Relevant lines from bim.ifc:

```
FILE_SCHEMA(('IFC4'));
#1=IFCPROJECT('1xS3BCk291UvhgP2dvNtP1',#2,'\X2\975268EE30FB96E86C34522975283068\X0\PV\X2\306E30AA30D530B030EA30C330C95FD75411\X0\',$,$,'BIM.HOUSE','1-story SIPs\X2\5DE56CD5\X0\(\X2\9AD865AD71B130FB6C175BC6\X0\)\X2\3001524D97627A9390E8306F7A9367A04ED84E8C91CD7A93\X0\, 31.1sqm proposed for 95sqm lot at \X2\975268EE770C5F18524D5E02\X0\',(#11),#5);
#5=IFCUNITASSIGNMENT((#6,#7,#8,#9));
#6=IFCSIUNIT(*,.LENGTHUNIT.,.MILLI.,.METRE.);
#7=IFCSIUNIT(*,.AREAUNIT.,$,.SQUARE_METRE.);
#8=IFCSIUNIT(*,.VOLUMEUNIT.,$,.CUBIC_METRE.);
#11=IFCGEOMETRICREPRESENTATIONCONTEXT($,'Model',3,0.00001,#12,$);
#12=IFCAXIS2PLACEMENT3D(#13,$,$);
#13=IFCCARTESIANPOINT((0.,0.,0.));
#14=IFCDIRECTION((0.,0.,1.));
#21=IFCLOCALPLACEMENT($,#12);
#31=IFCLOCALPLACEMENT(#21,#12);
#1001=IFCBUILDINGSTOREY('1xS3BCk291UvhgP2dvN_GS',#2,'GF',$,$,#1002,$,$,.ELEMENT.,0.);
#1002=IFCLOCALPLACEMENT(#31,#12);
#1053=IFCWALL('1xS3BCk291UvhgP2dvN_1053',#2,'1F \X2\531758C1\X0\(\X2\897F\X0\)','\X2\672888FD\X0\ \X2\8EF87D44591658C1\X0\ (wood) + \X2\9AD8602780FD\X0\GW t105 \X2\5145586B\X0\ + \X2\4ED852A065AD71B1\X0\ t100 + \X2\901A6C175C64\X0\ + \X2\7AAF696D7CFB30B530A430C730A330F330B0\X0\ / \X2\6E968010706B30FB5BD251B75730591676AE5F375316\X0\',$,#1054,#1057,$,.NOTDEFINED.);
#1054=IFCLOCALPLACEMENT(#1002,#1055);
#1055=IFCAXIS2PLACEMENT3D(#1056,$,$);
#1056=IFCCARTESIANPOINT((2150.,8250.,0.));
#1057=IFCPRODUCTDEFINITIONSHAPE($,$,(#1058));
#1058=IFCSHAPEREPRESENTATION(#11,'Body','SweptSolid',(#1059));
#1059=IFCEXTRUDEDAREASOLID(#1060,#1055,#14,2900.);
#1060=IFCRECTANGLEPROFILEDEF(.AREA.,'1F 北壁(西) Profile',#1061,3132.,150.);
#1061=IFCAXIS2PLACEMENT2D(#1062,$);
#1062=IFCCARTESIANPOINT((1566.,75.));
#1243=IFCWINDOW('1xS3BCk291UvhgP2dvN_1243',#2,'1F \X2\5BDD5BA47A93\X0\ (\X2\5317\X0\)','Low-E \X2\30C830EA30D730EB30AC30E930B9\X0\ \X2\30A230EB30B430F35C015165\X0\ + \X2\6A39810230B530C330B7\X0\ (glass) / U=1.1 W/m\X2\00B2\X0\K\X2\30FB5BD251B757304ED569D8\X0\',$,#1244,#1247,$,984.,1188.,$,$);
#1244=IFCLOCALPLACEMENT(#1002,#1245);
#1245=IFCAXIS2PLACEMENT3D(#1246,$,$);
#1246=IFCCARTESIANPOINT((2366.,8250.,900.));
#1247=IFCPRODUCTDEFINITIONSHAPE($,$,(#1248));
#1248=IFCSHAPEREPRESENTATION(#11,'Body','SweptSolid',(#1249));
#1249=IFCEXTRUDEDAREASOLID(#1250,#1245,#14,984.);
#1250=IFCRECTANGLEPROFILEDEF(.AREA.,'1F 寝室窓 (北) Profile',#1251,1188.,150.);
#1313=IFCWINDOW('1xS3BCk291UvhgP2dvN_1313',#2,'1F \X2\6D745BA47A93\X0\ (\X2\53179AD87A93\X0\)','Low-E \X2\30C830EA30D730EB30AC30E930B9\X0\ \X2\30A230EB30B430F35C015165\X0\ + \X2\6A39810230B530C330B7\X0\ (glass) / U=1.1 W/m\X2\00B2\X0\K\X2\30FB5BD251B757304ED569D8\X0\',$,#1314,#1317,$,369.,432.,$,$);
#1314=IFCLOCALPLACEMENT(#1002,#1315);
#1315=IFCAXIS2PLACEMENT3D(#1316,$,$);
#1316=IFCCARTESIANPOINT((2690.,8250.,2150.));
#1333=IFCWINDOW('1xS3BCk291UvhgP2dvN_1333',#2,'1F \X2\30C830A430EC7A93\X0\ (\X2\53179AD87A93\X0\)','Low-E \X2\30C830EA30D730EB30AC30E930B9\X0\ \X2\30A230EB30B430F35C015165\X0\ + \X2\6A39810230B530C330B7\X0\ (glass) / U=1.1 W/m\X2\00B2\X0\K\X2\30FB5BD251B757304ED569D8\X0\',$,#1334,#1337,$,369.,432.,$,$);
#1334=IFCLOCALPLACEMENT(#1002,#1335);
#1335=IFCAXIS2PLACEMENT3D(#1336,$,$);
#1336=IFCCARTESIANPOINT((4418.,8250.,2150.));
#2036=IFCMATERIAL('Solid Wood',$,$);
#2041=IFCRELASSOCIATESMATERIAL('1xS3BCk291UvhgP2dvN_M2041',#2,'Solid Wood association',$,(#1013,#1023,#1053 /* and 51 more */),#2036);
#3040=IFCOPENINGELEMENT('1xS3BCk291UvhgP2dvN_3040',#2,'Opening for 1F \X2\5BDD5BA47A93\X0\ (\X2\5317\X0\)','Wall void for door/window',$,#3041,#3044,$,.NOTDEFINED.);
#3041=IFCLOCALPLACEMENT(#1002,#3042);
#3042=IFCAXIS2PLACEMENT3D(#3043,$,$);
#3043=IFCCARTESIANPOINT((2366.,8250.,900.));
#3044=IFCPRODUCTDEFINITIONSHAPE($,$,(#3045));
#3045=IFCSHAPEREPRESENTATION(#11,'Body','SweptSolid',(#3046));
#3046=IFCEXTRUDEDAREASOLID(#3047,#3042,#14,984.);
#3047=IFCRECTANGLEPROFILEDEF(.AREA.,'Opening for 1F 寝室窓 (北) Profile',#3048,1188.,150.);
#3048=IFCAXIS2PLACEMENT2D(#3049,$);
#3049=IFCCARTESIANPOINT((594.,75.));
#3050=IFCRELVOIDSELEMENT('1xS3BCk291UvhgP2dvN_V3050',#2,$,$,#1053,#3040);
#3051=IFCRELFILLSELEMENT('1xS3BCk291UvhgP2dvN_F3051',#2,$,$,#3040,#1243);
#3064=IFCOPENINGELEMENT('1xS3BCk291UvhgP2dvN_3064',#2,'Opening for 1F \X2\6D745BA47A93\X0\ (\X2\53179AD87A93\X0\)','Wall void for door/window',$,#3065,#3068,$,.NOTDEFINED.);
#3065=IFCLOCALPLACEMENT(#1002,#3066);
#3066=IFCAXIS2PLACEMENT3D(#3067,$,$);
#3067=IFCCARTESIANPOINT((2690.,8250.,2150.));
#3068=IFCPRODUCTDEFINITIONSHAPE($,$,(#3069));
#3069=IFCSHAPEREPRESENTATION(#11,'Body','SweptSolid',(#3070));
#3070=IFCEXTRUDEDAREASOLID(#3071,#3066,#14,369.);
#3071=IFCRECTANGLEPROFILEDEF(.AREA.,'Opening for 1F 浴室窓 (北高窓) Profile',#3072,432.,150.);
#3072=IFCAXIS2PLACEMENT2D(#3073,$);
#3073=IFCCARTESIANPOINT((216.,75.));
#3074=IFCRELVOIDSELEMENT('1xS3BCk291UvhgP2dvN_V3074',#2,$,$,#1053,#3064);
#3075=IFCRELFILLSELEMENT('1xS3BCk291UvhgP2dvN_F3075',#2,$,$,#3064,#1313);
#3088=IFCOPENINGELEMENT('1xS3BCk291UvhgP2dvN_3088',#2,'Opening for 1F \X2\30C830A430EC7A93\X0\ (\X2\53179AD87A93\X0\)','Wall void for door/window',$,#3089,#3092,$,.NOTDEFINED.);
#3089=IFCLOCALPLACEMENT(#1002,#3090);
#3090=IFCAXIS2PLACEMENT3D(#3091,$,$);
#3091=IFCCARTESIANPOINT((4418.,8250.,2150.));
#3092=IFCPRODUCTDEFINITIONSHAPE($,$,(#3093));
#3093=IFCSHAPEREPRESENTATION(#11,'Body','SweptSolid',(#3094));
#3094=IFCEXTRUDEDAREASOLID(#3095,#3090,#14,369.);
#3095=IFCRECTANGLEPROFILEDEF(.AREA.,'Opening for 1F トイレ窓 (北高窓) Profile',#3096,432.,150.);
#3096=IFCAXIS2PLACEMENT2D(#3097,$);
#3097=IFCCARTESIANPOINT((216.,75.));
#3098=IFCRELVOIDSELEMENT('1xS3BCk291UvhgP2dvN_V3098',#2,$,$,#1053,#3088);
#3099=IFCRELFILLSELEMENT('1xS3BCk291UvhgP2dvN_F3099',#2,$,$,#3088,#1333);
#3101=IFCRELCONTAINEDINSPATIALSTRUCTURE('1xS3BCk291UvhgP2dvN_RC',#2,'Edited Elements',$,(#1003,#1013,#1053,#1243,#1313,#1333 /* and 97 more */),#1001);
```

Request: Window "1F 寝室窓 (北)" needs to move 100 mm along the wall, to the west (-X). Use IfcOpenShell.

```python
import ifcopenshell
import ifcopenshell.api.geometry
import ifcopenshell.util.placement
import ifcopenshell.util.unit

model = ifcopenshell.open("bim.ifc")
unit_scale = ifcopenshell.util.unit.calculate_unit_scale(model)

window = model.by_guid("1xS3BCk291UvhgP2dvN_1243")
opening = window.FillsVoids[0].RelatingOpeningElement
wall = opening.VoidsElements[0].RelatingBuildingElement

wall_matrix = ifcopenshell.util.placement.get_local_placement(wall.ObjectPlacement)
shift = wall_matrix[:3, 0] * -0.1 / unit_scale
before = ifcopenshell.util.placement.get_local_placement(window.ObjectPlacement)[:3, 3].copy()

# The window is not placed relative to its opening, so move both.
for product in (opening, window):
    matrix = ifcopenshell.util.placement.get_local_placement(product.ObjectPlacement)
    matrix[:3, 3] += shift
    ifcopenshell.api.geometry.edit_object_placement(model, product=product, matrix=matrix, is_si=False)

after = ifcopenshell.util.placement.get_local_placement(window.ObjectPlacement)[:3, 3]
print("window moved by", (after - before).round(3) + 0.0)

model.write("bim_v2.ifc")
```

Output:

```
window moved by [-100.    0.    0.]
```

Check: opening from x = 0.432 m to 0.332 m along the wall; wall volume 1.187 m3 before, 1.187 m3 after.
